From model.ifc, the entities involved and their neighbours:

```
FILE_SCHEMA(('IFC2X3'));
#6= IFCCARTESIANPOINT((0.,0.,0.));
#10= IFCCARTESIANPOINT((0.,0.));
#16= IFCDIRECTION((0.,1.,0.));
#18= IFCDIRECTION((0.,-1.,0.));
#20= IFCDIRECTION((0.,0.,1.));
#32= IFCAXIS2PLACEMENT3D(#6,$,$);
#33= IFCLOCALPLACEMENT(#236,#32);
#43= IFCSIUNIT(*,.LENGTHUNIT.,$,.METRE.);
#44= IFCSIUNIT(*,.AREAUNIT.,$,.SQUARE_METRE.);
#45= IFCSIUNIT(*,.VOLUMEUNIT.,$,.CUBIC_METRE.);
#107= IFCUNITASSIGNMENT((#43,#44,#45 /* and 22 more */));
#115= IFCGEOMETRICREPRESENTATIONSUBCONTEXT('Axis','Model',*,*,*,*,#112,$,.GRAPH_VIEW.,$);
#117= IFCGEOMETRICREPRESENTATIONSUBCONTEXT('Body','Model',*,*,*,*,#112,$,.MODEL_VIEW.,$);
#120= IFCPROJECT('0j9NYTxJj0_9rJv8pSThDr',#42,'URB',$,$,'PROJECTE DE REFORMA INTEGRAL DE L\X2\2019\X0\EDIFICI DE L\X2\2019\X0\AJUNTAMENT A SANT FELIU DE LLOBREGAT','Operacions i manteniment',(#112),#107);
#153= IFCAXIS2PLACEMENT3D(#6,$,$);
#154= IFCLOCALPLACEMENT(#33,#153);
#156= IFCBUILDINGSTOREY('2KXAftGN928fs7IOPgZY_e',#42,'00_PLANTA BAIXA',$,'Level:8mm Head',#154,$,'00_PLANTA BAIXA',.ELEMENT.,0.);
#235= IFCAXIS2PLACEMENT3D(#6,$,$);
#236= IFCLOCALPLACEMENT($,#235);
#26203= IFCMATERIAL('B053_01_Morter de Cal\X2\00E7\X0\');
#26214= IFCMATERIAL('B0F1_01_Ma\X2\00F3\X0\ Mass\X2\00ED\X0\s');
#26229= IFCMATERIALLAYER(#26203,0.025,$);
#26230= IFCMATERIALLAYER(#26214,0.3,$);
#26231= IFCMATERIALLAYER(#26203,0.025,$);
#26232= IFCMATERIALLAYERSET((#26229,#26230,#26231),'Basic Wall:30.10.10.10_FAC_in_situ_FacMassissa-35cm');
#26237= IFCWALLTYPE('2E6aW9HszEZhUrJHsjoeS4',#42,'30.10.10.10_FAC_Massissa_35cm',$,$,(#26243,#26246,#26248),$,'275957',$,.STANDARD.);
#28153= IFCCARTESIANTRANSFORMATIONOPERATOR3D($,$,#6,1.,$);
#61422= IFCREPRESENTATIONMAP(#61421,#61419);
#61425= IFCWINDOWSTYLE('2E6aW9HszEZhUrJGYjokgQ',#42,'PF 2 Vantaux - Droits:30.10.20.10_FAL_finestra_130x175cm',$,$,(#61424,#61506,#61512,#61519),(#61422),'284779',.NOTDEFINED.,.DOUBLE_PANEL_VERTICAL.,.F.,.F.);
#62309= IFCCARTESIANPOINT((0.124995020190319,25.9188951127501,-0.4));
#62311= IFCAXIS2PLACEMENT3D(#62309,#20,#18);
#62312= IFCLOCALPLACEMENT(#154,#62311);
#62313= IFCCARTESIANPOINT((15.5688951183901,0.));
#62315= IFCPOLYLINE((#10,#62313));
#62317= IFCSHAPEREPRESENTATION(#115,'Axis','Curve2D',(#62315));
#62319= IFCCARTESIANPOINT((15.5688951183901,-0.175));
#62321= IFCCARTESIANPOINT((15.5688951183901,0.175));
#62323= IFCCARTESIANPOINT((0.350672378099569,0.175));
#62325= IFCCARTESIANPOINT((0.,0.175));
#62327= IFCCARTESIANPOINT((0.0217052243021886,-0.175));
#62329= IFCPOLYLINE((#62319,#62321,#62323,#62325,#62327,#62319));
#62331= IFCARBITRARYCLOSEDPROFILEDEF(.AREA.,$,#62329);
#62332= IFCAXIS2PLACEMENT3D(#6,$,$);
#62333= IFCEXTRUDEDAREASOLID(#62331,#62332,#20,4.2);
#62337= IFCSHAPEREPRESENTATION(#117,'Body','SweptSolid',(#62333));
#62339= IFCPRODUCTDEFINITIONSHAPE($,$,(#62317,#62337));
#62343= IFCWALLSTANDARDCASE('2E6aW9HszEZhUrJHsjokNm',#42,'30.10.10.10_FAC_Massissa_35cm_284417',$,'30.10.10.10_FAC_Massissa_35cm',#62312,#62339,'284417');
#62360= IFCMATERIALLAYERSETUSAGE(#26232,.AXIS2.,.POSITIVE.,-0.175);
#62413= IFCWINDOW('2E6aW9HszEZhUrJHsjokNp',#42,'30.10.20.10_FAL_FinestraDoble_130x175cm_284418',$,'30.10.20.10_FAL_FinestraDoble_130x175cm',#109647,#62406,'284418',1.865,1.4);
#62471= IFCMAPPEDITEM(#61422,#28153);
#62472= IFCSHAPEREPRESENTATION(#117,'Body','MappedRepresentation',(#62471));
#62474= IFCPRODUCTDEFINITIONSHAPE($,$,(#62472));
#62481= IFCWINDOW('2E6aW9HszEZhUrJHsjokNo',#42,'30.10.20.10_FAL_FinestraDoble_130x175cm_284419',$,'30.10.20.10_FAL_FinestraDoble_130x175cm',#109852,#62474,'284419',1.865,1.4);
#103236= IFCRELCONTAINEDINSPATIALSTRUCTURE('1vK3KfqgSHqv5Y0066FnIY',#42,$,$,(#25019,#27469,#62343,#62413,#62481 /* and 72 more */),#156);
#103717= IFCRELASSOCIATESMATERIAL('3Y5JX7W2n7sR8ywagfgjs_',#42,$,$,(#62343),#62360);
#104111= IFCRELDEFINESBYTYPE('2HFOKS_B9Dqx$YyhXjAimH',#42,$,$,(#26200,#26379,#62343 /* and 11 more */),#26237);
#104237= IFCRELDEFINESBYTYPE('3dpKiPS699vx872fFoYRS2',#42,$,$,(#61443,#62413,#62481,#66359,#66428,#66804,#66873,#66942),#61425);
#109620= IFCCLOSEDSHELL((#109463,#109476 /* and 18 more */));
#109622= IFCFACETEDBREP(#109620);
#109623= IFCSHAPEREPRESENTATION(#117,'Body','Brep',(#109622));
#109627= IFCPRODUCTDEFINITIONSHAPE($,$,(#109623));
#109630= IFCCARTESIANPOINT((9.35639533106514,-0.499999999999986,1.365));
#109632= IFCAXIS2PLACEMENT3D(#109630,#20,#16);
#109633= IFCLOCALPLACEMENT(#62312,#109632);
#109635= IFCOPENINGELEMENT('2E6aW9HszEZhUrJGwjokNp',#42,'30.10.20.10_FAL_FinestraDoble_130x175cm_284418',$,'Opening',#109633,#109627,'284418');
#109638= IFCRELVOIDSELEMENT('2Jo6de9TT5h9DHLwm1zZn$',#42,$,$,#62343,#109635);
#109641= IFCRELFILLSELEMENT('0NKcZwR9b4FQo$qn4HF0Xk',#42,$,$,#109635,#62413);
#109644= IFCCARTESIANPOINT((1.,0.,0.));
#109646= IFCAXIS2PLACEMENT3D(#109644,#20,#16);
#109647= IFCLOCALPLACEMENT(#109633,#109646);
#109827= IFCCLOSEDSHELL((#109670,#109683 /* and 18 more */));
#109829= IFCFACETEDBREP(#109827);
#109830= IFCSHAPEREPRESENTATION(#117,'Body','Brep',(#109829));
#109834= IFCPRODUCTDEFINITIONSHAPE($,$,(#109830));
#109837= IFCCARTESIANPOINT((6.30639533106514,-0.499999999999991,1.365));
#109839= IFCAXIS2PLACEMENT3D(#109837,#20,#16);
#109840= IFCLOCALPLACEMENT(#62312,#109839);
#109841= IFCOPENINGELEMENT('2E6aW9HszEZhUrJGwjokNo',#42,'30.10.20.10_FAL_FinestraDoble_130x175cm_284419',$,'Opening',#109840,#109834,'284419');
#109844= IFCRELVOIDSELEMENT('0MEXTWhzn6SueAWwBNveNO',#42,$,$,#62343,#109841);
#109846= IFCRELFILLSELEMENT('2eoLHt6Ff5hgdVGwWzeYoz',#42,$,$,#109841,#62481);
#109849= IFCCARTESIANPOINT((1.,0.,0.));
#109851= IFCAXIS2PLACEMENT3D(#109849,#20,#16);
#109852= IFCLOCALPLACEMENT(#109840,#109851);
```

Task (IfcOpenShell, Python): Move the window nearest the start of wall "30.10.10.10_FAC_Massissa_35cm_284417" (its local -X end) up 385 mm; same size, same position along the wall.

```python
import numpy as np
import ifcopenshell
import ifcopenshell.api.geometry
import ifcopenshell.util.placement
import ifcopenshell.util.unit

model = ifcopenshell.open("model.ifc")
unit_scale = ifcopenshell.util.unit.calculate_unit_scale(model)

window = model.by_guid("2E6aW9HszEZhUrJHsjokNo")
opening = window.FillsVoids[0].RelatingOpeningElement
dz = 0.385 / unit_scale

shift = np.array([0.0, 0.0, dz])
# The window is placed relative to its opening, so it follows when the opening moves.
matrix = ifcopenshell.util.placement.get_local_placement(opening.ObjectPlacement)
matrix[:3, 3] += shift
ifcopenshell.api.geometry.edit_object_placement(
    model, product=opening, matrix=matrix, is_si=False, should_transform_children=True
)

print(f"moved by {dz * unit_scale:+.3f} m")

model.write("model_edited.ifc")
```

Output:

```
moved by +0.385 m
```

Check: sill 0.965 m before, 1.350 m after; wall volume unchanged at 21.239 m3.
